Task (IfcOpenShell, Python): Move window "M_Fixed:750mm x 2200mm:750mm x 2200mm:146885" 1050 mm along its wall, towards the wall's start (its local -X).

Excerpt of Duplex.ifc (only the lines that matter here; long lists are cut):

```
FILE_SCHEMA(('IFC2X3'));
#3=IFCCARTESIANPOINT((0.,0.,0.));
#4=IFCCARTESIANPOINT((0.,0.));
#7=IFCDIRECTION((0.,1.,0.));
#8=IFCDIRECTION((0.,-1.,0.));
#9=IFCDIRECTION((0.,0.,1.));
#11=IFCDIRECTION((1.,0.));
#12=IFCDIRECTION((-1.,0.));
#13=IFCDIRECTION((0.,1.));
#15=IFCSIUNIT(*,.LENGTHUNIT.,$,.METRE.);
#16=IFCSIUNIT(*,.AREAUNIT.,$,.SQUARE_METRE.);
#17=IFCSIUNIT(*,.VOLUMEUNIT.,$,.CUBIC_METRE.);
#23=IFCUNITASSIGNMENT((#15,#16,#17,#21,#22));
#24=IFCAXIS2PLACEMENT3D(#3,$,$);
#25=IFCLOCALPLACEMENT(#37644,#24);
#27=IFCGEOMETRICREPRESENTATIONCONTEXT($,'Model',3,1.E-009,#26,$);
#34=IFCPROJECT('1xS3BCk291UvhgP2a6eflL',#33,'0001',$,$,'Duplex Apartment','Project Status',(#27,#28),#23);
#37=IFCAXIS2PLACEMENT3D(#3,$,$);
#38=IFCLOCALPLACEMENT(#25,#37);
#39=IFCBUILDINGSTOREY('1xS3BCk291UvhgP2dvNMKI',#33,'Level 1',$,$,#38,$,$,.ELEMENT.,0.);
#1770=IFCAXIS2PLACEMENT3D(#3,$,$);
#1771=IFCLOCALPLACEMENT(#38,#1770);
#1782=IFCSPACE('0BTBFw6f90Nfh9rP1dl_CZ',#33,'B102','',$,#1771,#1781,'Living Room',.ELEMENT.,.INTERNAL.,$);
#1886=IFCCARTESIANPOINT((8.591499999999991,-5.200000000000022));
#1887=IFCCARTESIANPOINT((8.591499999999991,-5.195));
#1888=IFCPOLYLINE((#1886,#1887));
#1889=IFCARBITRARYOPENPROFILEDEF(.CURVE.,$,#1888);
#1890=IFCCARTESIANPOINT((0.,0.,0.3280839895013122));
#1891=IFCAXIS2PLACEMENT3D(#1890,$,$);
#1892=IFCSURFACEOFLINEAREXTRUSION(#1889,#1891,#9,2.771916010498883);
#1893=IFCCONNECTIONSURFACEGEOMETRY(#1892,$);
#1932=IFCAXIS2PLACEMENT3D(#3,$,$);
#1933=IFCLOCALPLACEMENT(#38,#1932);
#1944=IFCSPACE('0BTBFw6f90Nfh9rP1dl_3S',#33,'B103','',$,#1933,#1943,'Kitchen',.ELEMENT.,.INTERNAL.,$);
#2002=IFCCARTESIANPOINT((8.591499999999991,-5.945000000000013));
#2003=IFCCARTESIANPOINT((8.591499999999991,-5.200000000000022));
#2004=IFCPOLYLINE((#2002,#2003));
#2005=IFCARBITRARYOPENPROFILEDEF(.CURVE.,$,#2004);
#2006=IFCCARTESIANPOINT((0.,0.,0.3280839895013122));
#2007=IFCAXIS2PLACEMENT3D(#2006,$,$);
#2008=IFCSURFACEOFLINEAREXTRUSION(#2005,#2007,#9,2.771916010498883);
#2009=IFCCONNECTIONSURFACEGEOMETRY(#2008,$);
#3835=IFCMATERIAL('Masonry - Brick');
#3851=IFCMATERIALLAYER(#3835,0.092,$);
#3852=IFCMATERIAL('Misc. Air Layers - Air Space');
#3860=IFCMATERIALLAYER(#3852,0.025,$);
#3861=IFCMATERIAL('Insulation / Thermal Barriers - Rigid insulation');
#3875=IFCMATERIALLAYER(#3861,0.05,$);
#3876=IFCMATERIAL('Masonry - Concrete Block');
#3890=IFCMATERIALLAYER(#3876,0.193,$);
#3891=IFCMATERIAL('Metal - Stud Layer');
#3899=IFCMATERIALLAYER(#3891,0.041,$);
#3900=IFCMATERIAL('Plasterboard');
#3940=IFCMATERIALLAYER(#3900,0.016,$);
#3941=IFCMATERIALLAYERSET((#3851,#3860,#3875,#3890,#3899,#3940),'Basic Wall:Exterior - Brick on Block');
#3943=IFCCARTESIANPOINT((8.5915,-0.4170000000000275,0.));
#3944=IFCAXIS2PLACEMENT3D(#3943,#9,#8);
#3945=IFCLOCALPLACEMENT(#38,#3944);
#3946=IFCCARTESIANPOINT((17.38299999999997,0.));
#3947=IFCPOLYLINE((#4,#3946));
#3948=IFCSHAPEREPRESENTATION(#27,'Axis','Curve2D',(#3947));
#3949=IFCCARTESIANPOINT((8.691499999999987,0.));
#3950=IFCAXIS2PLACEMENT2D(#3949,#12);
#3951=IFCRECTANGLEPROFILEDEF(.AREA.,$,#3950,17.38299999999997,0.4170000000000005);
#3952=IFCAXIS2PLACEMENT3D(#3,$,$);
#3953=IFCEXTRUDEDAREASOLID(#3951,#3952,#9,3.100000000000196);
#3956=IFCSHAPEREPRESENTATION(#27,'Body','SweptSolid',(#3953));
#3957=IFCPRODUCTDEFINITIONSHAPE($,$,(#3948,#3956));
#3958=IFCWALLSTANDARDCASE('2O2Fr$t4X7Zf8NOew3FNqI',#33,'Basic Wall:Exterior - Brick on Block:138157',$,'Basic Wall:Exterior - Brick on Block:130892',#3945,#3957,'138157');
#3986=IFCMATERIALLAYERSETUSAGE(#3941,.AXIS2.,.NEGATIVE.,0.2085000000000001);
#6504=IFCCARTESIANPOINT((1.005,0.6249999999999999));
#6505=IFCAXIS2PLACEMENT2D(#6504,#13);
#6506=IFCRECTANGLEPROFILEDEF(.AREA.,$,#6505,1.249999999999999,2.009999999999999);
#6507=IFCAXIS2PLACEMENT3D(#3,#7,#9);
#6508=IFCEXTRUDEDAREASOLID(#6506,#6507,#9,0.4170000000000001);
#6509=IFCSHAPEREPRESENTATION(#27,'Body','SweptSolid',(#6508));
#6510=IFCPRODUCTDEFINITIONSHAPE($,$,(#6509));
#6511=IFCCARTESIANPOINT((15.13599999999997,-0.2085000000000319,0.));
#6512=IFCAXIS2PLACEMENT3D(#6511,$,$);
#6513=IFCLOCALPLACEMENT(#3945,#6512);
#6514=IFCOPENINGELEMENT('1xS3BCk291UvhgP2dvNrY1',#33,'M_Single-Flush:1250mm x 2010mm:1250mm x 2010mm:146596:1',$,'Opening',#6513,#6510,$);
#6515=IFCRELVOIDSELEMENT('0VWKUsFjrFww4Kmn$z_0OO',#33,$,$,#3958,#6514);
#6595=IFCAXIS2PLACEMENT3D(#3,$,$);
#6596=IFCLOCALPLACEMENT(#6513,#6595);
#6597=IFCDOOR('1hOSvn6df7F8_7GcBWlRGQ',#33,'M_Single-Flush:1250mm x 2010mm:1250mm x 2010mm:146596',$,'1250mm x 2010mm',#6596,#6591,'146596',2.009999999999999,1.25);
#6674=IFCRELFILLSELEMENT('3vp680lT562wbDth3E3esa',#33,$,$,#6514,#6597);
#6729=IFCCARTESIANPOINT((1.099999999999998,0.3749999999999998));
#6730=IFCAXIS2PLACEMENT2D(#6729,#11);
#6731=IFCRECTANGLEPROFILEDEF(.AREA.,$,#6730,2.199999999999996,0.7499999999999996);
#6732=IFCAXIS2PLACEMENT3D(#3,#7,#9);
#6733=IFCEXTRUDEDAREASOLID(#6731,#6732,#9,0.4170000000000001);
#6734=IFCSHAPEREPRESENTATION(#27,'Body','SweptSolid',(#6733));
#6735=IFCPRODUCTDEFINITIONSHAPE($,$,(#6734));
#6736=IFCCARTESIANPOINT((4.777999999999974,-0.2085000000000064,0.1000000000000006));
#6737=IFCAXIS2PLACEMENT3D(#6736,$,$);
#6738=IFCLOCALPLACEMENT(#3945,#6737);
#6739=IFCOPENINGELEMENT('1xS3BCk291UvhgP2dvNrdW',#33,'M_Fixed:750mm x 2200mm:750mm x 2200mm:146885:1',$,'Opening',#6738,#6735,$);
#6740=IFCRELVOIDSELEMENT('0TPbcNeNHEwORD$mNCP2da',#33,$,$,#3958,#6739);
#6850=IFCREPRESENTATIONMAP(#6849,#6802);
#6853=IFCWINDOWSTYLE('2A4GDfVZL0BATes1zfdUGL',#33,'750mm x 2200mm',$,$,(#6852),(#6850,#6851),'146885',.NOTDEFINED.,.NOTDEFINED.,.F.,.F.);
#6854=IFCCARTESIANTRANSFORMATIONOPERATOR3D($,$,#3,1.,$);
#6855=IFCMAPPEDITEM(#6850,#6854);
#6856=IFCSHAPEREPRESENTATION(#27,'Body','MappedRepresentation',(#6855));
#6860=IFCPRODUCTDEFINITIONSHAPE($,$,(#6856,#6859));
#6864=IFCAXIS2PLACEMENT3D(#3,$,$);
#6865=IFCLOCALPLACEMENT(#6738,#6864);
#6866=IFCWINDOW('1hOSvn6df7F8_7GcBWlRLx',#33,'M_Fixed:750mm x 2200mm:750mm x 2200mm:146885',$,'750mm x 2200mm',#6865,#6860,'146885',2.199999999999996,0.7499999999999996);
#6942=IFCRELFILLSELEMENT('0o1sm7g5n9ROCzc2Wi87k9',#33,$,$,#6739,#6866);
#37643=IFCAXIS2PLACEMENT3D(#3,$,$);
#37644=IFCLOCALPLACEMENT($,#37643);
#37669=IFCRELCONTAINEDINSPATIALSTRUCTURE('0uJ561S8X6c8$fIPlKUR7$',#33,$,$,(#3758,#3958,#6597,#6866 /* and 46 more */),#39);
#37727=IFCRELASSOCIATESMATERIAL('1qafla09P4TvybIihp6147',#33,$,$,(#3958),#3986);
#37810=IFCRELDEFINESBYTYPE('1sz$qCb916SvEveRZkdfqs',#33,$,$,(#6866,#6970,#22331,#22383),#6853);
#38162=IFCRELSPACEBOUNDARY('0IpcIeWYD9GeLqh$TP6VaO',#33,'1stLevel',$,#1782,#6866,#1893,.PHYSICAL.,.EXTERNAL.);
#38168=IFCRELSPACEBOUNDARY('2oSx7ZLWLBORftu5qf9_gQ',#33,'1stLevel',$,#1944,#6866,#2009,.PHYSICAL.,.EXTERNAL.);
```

```python
import numpy as np
import ifcopenshell
import ifcopenshell.api.geometry
import ifcopenshell.util.placement

model = ifcopenshell.open("Duplex.ifc")

window = model.by_guid("1hOSvn6df7F8_7GcBWlRLx")
opening = window.FillsVoids[0].RelatingOpeningElement
wall = opening.VoidsElements[0].RelatingBuildingElement

wall_matrix = ifcopenshell.util.placement.get_local_placement(wall.ObjectPlacement)
shift = wall_matrix[:3, 0] * -1.05
before = ifcopenshell.util.placement.get_local_placement(window.ObjectPlacement)[:3, 3].copy()

# The window is placed relative to its opening, so it follows when the opening moves.
matrix = ifcopenshell.util.placement.get_local_placement(opening.ObjectPlacement)
matrix[:3, 3] += shift
ifcopenshell.api.geometry.edit_object_placement(
    model, product=opening, matrix=matrix, is_si=False, should_transform_children=True
)

# Space boundary surfaces are stored in each space's coordinates; move them too.
for rel in window.ProvidesBoundaries:
    if not rel.ConnectionGeometry:
        continue
    surface = rel.ConnectionGeometry.SurfaceOnRelatingElement
    space_matrix = ifcopenshell.util.placement.get_local_placement(rel.RelatingSpace.ObjectPlacement)
    point = np.array(surface.Position.Location.Coordinates) + space_matrix[:3, :3].T @ shift
    surface.Position = model.createIfcAxis2Placement3D(
        model.createIfcCartesianPoint(point.tolist()), surface.Position.Axis, surface.Position.RefDirection
    )

after = ifcopenshell.util.placement.get_local_placement(window.ObjectPlacement)[:3, 3]
print("window moved by", (after - before).round(3) + 0.0)

model.write("Duplex_updated.ifc")
```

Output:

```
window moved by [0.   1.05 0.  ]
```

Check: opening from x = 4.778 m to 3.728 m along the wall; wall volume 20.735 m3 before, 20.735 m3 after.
